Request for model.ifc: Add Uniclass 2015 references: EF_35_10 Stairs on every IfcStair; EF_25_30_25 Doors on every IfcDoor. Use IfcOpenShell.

First a look at what the model holds.

```python
import ifcopenshell

model = ifcopenshell.open("model.ifc")
print(model.schema)
print("classifications:", [c.Name for c in model.by_type("IfcClassification")])
for ifc_class in ("IfcDoor", "IfcRoof", "IfcStair", "IfcWall", "IfcWindow"):
    print(ifc_class, len(model.by_type(ifc_class)))
```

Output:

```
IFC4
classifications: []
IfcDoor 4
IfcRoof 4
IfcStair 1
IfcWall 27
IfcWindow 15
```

```python
import ifcopenshell
import ifcopenshell.api.classification

model = ifcopenshell.open("model.ifc")

system = ifcopenshell.api.classification.add_classification(model, classification="Uniclass 2015")

codes = {
    "IfcStair": ("EF_35_10", "Stairs"),
    "IfcDoor": ("EF_25_30_25", "Doors"),
}
for ifc_class, (code, name) in codes.items():
    products = model.by_type(ifc_class)
    ifcopenshell.api.classification.add_reference(
        model, products=products, classification=system, identification=code, name=name
    )
    print(code, len(products))

model.write("model_rev.ifc")
```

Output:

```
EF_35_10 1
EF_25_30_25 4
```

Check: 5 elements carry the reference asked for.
